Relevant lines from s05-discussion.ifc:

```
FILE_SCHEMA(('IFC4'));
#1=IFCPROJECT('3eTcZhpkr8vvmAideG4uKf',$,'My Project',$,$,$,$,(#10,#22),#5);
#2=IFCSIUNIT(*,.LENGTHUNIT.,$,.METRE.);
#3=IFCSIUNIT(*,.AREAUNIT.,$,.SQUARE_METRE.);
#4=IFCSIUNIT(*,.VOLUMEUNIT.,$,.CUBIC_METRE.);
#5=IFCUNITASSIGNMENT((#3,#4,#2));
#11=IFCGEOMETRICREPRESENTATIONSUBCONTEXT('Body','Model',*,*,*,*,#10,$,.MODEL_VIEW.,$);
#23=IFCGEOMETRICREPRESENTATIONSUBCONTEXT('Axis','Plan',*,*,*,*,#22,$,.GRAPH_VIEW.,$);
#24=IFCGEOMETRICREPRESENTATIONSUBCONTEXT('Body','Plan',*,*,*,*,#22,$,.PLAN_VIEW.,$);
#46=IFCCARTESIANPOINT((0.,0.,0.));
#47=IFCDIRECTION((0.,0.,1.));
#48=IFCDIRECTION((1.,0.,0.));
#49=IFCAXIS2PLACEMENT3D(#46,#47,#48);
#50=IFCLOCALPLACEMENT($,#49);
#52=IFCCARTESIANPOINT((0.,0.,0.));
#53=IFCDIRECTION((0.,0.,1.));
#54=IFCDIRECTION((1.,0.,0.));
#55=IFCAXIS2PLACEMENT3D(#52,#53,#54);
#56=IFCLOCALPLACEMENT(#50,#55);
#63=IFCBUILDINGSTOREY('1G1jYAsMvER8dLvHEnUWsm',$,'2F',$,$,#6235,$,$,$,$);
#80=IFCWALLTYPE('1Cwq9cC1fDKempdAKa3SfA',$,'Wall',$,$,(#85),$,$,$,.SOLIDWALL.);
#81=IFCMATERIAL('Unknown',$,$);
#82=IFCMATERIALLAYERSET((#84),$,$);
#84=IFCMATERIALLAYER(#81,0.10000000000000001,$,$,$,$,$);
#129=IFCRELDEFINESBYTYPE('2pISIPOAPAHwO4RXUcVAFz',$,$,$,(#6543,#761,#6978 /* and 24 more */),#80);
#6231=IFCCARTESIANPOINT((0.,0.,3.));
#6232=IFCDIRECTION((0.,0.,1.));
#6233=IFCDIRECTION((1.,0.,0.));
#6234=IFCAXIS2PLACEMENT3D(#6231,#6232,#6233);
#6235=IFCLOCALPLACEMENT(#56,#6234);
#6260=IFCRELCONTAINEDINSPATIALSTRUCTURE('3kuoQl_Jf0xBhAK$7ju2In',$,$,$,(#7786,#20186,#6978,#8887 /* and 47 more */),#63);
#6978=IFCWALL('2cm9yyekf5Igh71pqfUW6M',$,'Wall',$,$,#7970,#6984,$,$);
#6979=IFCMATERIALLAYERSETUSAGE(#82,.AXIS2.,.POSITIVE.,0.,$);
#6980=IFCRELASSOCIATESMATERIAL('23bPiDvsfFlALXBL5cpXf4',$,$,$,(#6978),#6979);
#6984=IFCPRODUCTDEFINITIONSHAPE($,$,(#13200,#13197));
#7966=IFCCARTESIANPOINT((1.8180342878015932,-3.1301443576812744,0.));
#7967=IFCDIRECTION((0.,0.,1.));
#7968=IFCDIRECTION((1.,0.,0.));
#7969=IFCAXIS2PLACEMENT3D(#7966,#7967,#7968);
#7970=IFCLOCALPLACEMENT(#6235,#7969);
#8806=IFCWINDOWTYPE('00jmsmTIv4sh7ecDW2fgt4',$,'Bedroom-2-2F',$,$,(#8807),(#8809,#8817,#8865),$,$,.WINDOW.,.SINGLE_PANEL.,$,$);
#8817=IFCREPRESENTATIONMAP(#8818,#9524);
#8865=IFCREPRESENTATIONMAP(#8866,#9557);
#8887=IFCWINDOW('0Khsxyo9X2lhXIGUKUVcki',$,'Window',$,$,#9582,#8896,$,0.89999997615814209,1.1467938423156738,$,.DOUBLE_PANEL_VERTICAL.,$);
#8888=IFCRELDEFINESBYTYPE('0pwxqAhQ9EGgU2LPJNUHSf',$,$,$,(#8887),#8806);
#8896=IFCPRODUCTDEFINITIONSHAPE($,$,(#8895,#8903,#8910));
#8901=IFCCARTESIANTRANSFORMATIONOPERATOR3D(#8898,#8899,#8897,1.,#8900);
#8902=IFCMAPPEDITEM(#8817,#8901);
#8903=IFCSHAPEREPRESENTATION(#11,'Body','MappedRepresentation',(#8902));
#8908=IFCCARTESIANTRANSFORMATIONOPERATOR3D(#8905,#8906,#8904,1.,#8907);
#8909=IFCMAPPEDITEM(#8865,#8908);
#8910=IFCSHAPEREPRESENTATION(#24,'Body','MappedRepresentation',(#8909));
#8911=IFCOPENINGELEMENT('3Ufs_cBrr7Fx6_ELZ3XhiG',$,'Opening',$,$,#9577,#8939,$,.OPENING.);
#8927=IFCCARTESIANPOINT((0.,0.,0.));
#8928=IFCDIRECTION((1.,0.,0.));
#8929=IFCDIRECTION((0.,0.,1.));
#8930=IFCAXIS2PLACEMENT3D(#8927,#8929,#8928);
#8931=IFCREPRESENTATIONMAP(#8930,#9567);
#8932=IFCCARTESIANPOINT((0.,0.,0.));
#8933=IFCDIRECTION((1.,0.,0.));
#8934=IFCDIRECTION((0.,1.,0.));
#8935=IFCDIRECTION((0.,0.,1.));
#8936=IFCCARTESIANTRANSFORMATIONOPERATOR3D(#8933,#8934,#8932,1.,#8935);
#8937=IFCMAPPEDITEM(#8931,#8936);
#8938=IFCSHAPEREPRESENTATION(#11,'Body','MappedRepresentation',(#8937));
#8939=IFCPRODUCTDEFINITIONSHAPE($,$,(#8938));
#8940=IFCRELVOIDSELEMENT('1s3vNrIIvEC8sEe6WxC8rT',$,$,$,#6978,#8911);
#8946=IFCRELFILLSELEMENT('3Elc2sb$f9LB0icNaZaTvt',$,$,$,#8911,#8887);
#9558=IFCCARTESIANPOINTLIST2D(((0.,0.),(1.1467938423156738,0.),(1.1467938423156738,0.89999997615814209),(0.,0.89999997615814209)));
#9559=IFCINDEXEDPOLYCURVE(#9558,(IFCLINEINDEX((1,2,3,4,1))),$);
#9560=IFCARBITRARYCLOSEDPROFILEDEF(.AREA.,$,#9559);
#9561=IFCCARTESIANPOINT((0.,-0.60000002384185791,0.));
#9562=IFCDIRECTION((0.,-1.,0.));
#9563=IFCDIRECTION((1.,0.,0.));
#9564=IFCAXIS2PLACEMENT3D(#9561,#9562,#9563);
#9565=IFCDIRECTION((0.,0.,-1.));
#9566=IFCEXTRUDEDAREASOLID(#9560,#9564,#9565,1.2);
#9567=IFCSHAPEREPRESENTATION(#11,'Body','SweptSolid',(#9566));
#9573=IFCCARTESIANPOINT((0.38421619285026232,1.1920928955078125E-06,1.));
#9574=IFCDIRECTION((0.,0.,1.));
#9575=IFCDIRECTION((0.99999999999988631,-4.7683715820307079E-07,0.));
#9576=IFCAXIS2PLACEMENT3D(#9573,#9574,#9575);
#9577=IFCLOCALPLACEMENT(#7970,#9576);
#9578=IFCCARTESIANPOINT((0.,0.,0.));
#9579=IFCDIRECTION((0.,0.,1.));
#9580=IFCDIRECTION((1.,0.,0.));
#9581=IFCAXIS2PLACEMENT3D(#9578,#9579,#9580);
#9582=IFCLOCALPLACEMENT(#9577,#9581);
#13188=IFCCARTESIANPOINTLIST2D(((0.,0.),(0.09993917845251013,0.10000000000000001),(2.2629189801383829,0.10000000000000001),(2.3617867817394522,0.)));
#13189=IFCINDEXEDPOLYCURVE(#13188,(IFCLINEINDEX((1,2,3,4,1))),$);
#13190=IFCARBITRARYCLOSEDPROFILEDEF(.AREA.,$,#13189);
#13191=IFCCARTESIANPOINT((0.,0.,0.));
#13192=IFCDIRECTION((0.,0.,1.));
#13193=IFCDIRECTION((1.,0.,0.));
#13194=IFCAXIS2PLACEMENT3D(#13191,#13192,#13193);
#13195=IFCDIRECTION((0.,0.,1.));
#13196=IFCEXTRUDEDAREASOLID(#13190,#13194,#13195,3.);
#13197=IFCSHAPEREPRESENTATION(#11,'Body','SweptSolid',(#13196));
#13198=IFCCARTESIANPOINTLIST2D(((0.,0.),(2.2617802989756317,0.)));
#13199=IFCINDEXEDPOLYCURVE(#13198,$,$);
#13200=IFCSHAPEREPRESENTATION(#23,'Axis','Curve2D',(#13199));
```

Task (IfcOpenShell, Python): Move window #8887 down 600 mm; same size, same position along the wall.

```python
import numpy as np
import ifcopenshell
import ifcopenshell.api.geometry
import ifcopenshell.util.placement
import ifcopenshell.util.unit

model = ifcopenshell.open("s05-discussion.ifc")
unit_scale = ifcopenshell.util.unit.calculate_unit_scale(model)

window = model.by_id(8887)
opening = window.FillsVoids[0].RelatingOpeningElement
dz = -0.6 / unit_scale

shift = np.array([0.0, 0.0, dz])
# The window is placed relative to its opening, so it follows when the opening moves.
matrix = ifcopenshell.util.placement.get_local_placement(opening.ObjectPlacement)
matrix[:3, 3] += shift
ifcopenshell.api.geometry.edit_object_placement(
    model, product=opening, matrix=matrix, is_si=False, should_transform_children=True
)

print(f"moved by {dz * unit_scale:+.3f} m")

model.write("s05-discussion_updated.ifc")
```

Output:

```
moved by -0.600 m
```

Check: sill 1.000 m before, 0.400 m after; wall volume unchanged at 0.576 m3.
